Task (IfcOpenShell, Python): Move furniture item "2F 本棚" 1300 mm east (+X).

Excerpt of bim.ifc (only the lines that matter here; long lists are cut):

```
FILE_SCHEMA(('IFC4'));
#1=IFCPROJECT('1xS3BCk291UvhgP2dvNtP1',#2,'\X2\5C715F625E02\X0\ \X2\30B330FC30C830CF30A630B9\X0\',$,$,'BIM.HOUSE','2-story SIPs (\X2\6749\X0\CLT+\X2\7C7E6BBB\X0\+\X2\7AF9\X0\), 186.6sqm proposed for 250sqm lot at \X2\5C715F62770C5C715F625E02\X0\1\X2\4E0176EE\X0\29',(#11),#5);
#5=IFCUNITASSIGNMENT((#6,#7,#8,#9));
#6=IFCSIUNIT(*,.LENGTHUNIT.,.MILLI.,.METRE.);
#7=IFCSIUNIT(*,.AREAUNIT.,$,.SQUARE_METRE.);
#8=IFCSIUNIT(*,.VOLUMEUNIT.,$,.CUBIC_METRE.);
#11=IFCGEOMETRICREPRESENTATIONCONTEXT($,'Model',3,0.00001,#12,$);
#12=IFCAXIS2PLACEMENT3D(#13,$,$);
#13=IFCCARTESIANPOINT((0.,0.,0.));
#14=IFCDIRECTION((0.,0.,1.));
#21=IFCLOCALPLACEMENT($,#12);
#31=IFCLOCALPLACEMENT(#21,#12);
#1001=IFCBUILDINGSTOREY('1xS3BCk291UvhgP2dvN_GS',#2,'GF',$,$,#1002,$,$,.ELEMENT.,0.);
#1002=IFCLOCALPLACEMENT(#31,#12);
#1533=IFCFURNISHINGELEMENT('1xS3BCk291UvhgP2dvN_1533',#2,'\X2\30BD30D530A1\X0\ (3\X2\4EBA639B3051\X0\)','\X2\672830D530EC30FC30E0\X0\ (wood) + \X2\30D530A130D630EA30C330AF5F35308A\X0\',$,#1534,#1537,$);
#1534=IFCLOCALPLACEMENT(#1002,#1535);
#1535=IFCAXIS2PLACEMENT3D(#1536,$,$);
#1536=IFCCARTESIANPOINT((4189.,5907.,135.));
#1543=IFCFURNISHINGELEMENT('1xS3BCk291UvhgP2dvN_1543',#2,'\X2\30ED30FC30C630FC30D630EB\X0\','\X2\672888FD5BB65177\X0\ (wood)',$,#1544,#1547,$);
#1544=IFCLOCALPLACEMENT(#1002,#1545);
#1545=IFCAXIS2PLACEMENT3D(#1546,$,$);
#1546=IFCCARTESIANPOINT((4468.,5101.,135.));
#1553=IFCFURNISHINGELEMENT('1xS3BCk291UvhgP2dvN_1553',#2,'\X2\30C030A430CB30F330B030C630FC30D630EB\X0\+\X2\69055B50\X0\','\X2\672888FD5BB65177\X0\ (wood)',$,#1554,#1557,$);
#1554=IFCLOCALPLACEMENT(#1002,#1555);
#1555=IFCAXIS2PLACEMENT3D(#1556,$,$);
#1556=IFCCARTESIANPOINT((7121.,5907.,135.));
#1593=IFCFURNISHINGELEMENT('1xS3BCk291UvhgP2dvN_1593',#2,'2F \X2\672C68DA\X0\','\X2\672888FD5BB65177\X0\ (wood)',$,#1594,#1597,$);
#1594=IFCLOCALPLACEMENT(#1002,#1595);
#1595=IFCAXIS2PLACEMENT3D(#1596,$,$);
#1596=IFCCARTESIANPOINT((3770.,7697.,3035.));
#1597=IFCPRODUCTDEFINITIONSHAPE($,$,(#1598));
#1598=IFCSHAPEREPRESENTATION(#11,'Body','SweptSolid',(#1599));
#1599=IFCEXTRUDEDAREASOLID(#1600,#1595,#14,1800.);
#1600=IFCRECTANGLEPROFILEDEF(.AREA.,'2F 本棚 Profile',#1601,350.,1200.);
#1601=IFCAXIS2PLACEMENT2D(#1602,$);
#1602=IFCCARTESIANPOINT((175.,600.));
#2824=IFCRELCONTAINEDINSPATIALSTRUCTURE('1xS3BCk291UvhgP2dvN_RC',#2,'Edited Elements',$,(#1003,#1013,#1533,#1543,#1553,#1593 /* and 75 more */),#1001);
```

```python
import ifcopenshell
import ifcopenshell.api.geometry
import ifcopenshell.util.placement

model = ifcopenshell.open("bim.ifc")

item = model.by_guid("1xS3BCk291UvhgP2dvN_1593")
matrix = ifcopenshell.util.placement.get_local_placement(item.ObjectPlacement)
matrix[0, 3] += 1300.0
ifcopenshell.api.geometry.edit_object_placement(model, product=item, matrix=matrix, is_si=False)

print(ifcopenshell.util.placement.get_local_placement(item.ObjectPlacement).round(3) + 0.0)

model.write("bim_updated.ifc")
```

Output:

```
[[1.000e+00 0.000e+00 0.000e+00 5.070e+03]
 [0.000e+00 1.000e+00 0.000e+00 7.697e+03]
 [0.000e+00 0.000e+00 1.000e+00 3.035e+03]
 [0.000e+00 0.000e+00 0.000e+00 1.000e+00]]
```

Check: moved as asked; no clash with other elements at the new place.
